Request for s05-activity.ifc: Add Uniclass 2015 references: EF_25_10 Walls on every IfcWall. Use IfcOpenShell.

First a look at what the model holds.

```python
import ifcopenshell

model = ifcopenshell.open("s05-activity.ifc")
print(model.schema)
print("classifications:", [c.Name for c in model.by_type("IfcClassification")])
for ifc_class in ("IfcDoor", "IfcRoof", "IfcStair", "IfcWall", "IfcWindow"):
    print(ifc_class, len(model.by_type(ifc_class)))
```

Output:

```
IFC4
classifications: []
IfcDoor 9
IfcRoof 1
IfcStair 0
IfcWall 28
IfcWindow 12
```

```python
import ifcopenshell
import ifcopenshell.api.classification

model = ifcopenshell.open("s05-activity.ifc")

system = ifcopenshell.api.classification.add_classification(model, classification="Uniclass 2015")

codes = {
    "IfcWall": ("EF_25_10", "Walls"),
}
for ifc_class, (code, name) in codes.items():
    products = model.by_type(ifc_class)
    ifcopenshell.api.classification.add_reference(
        model, products=products, classification=system, identification=code, name=name
    )
    print(code, len(products))

model.write("s05-activity_rev.ifc")
```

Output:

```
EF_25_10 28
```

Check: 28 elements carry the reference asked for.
